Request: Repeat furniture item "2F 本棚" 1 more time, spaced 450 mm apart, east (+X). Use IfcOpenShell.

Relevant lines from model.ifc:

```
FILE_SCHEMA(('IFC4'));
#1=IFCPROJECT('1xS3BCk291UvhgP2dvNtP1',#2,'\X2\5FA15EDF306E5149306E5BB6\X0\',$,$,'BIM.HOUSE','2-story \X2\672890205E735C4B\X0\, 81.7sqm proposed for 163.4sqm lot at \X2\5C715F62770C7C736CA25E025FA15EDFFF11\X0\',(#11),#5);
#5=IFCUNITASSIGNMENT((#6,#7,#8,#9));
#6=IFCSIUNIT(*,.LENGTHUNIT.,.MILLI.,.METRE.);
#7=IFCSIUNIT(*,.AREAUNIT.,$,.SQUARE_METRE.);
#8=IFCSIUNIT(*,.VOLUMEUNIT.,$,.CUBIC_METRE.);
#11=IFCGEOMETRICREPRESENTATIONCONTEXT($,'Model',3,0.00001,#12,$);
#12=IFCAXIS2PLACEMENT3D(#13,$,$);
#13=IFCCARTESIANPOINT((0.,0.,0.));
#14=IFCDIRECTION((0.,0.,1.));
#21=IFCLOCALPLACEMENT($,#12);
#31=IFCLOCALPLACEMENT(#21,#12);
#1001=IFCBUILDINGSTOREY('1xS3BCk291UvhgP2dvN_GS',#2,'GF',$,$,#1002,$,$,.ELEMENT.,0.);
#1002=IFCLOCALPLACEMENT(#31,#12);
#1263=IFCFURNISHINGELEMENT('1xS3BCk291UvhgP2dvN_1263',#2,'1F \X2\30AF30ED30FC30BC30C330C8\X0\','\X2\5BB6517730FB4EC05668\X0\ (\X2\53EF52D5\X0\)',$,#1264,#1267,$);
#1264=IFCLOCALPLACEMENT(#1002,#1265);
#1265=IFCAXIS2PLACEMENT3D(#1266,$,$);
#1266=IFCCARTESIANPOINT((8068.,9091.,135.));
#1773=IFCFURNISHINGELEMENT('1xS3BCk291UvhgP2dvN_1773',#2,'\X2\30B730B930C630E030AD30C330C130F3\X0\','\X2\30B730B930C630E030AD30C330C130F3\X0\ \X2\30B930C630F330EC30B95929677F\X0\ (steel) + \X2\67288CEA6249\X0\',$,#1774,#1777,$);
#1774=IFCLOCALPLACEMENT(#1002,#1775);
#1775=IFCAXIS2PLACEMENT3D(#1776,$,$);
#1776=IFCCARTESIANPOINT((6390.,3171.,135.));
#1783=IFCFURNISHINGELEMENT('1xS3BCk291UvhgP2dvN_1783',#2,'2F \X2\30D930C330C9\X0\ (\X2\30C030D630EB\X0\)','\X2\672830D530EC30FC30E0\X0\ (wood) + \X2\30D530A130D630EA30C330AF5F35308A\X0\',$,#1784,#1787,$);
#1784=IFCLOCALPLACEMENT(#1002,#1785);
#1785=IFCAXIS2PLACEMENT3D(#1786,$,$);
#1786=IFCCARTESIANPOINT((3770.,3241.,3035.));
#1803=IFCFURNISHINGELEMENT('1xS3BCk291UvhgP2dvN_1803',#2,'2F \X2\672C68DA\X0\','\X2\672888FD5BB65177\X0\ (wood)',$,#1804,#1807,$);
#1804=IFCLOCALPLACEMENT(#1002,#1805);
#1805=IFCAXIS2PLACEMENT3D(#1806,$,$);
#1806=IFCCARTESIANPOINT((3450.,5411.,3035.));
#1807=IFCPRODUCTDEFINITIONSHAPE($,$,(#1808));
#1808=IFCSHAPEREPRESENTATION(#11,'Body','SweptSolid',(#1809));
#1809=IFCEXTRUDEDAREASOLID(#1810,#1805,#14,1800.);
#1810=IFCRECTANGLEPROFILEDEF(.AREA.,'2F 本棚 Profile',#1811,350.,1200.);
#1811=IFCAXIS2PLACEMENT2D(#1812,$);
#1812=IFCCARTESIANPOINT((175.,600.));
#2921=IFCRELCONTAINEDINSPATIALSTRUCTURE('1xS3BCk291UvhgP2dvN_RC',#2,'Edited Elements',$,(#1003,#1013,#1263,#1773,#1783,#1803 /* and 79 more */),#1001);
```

```python
import numpy as np
import ifcopenshell
import ifcopenshell.api.geometry
import ifcopenshell.api.root
import ifcopenshell.util.element
import ifcopenshell.util.placement

model = ifcopenshell.open("model.ifc")


def reuse_history(source, copy):
    """copy_class also copies each property set's owner history, people and application; keep the originals."""
    for rel in copy.IsDefinedBy:
        if rel.is_a("IfcRelDefinesByProperties") and (history := rel.RelatingPropertyDefinition.OwnerHistory):
            rel.RelatingPropertyDefinition.OwnerHistory = source.OwnerHistory
            ifcopenshell.util.element.remove_deep2(model, history)


source = model.by_guid("1xS3BCk291UvhgP2dvN_1803")
base = ifcopenshell.util.placement.get_local_placement(source.ObjectPlacement)
step = np.array([1.0, 0.0, 0.0]) * 450.0

for i in range(1, 2):
    copy = ifcopenshell.api.root.copy_class(model, product=source)
    copy.Representation = ifcopenshell.util.element.copy_deep(
        model, source.Representation, exclude=["IfcGeometricRepresentationContext", "IfcRepresentationMap"]
    )
    reuse_history(source, copy)
    matrix = base.copy()
    matrix[:3, 3] += i * step
    print("added at", matrix[:3, 3].round(3) + 0.0)
    ifcopenshell.api.geometry.edit_object_placement(model, product=copy, matrix=matrix, is_si=False)

model.write("model_rev.ifc")
```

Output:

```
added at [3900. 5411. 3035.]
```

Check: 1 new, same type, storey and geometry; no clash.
